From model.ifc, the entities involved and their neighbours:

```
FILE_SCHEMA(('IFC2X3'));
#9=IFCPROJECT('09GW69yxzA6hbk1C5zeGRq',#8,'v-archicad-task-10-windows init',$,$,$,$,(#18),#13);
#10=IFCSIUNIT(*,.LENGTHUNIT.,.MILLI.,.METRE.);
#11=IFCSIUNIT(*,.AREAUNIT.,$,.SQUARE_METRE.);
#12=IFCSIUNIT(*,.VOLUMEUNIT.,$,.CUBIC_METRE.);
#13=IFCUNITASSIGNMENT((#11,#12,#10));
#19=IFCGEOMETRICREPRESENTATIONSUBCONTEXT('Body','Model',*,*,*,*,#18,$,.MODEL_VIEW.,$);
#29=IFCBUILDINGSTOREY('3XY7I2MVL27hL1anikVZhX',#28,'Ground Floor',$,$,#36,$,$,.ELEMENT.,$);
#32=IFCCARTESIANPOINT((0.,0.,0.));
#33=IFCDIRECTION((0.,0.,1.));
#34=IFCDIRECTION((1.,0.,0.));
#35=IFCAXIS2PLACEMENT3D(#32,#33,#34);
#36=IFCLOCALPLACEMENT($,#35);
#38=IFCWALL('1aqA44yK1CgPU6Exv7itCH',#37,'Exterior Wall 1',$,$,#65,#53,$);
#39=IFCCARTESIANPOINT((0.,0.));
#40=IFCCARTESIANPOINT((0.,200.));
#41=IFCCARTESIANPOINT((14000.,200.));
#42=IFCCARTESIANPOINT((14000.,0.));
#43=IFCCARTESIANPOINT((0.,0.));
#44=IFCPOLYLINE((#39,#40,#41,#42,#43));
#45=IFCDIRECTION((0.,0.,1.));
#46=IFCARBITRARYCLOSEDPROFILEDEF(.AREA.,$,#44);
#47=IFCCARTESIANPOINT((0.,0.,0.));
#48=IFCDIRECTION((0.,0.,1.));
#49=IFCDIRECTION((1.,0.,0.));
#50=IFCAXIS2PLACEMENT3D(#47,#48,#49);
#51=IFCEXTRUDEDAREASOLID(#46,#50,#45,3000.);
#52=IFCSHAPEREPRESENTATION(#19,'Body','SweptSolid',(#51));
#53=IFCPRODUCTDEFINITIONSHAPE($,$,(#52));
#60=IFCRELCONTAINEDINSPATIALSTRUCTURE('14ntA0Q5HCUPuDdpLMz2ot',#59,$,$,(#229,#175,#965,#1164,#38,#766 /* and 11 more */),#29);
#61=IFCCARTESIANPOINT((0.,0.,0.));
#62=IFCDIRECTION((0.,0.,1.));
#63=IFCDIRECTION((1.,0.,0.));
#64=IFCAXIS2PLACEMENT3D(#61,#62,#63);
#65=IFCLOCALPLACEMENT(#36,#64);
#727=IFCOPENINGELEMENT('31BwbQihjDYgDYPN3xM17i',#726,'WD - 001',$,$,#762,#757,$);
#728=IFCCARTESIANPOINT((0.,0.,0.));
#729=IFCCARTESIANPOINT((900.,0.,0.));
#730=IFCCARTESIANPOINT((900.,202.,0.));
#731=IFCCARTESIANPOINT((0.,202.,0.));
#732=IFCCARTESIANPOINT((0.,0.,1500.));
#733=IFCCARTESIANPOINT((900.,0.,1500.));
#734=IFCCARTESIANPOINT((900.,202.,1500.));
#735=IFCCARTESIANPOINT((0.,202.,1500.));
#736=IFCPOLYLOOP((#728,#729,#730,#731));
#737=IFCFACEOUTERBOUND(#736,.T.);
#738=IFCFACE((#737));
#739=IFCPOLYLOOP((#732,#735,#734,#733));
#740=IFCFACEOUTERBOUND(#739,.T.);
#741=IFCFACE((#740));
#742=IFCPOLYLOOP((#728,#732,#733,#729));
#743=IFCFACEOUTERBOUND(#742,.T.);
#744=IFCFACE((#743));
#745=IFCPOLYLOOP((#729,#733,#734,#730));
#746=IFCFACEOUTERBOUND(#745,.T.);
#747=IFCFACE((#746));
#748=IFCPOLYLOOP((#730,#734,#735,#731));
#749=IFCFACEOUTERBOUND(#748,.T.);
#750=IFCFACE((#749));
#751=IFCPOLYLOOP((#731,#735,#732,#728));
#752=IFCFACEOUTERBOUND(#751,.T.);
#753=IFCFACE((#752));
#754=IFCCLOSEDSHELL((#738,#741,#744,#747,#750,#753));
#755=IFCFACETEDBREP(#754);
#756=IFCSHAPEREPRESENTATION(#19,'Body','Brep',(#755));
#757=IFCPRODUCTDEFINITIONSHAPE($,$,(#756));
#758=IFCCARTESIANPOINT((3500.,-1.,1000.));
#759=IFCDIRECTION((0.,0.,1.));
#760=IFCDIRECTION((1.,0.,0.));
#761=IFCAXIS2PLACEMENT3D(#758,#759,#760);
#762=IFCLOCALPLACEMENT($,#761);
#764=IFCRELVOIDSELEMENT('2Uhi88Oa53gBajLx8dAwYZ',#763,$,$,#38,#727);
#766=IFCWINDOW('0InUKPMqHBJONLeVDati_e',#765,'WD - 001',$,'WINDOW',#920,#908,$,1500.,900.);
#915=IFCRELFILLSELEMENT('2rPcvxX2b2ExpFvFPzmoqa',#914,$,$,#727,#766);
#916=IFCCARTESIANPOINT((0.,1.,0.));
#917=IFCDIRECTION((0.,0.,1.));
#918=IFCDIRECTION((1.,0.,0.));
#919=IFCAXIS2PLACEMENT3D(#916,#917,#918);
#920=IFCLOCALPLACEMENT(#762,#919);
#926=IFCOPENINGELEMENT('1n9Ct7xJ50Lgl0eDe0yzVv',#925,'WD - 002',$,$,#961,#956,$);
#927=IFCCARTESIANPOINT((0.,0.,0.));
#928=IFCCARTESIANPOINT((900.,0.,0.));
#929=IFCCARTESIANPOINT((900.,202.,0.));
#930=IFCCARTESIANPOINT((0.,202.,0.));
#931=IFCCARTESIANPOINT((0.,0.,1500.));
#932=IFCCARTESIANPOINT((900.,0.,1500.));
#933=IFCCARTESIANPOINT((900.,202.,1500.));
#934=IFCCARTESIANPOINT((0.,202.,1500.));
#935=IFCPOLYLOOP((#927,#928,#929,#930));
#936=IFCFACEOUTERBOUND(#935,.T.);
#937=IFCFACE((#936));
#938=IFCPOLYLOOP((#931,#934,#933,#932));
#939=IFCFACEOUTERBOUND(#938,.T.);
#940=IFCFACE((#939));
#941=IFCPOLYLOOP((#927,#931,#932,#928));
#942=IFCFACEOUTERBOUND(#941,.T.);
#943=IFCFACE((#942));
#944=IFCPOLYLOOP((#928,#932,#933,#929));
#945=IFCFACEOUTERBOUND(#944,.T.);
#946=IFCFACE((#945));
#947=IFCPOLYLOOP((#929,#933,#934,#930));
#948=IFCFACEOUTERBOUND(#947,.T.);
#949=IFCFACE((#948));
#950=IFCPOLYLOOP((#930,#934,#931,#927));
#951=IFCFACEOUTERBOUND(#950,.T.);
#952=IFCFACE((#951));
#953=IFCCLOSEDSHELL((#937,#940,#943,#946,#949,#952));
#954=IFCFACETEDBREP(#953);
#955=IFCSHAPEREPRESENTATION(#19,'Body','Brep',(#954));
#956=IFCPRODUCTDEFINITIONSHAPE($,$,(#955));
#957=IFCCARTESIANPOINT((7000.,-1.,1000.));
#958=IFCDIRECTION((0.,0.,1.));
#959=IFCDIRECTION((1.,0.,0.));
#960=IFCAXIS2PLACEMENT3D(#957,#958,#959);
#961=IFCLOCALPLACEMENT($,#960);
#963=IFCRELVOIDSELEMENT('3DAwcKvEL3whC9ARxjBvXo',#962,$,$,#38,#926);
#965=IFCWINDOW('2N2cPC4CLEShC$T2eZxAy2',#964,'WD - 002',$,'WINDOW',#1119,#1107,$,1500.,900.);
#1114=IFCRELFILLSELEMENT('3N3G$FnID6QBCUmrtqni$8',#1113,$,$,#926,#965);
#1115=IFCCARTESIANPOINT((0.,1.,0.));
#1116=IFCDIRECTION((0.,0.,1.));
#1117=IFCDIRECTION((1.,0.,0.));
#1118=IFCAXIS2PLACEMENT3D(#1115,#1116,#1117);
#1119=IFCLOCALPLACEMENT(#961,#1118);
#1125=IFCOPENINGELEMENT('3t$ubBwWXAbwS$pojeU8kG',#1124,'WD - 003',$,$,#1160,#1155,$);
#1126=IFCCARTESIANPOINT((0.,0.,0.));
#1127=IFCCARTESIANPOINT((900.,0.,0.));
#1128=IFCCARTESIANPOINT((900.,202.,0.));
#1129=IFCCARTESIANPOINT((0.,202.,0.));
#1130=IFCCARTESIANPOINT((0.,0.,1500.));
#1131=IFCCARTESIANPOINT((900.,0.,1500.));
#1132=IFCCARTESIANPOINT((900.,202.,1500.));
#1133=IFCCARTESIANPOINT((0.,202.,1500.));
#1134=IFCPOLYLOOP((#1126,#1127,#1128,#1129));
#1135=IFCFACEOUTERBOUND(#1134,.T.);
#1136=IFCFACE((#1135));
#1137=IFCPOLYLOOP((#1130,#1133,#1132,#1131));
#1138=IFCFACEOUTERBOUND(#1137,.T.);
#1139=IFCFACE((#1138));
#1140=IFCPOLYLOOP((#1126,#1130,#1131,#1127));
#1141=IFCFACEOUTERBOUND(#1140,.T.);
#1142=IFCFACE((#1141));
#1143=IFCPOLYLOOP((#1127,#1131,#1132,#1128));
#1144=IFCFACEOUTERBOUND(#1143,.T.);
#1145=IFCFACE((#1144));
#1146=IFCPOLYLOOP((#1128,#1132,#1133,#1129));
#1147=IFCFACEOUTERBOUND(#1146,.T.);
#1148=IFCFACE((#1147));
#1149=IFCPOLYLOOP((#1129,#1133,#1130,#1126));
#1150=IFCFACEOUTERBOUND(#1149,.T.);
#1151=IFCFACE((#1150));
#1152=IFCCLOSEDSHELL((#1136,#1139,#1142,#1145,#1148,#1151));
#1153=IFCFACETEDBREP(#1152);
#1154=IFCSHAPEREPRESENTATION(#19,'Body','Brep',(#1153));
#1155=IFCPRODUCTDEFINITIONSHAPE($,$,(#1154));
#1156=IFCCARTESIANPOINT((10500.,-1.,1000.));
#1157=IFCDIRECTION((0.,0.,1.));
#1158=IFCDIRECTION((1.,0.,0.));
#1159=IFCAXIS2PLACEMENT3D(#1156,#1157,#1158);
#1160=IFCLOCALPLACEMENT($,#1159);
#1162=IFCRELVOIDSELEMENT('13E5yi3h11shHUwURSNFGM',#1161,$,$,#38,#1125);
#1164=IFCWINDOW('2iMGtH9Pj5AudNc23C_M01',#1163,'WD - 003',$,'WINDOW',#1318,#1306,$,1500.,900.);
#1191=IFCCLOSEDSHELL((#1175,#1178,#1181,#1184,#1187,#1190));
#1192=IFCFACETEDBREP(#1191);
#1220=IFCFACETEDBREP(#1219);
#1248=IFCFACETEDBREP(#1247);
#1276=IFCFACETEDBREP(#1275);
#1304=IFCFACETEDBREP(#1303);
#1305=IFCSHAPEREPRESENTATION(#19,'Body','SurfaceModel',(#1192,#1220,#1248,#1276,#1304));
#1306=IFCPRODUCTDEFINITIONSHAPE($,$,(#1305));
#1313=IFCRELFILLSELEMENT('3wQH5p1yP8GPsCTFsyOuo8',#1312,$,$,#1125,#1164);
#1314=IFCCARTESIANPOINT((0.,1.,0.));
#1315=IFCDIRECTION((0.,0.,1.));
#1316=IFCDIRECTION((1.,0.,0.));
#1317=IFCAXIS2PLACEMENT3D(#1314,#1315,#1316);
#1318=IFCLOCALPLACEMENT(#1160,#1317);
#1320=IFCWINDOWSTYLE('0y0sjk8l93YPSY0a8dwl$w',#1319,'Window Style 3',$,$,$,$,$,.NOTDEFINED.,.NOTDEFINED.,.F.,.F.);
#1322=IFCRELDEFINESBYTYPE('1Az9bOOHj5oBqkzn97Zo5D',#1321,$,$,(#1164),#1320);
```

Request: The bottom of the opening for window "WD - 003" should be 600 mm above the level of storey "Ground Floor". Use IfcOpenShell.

```python
import numpy as np
import ifcopenshell
import ifcopenshell.api.geometry
import ifcopenshell.geom
import ifcopenshell.util.element
import ifcopenshell.util.placement
import ifcopenshell.util.shape
import ifcopenshell.util.unit

model = ifcopenshell.open("model.ifc")
unit_scale = ifcopenshell.util.unit.calculate_unit_scale(model)

window = model.by_guid("2iMGtH9Pj5AudNc23C_M01")
opening = window.FillsVoids[0].RelatingOpeningElement
storey = ifcopenshell.util.element.get_container(window, ifc_class="IfcBuildingStorey")
level = ifcopenshell.util.placement.get_local_placement(storey.ObjectPlacement)[2, 3]

# The opening's origin need not be at the sill, so measure its lowest point.
shape = ifcopenshell.geom.create_shape(ifcopenshell.geom.settings(), opening)
bottom = ifcopenshell.util.shape.get_shape_bottom_elevation(shape, shape.geometry) / unit_scale
dz = level + 0.6 / unit_scale - bottom

shift = np.array([0.0, 0.0, dz])
# The window is placed relative to its opening, so it follows when the opening moves.
matrix = ifcopenshell.util.placement.get_local_placement(opening.ObjectPlacement)
matrix[:3, 3] += shift
ifcopenshell.api.geometry.edit_object_placement(
    model, product=opening, matrix=matrix, is_si=False, should_transform_children=True
)

print(f"moved by {dz * unit_scale:+.3f} m")

model.write("model_updated.ifc")
```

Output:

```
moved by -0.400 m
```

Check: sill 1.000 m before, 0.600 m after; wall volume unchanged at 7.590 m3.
